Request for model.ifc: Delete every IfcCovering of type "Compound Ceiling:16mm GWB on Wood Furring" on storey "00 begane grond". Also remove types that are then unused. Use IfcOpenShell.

First a look at what the model holds.

```python
import ifcopenshell
import ifcopenshell.util.element

model = ifcopenshell.open("model.ifc")
print(model.schema)
storey = next(s for s in model.by_type("IfcBuildingStorey") if s.Name == "00 begane grond")
coverings = [e for e in ifcopenshell.util.element.get_decomposition(storey) if e.is_a("IfcCovering")]
seen = {}
for e in coverings:
    element_type = ifcopenshell.util.element.get_type(e)
    name = element_type.Name if element_type not in (None, e) else None
    seen[name] = seen.get(name, 0) + 1
for name, count in sorted(seen.items(), key=str):
    print(count, "x", name)
```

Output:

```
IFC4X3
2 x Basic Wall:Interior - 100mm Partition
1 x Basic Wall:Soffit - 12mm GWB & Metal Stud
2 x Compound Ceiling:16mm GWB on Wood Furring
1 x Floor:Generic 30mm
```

```python
import ifcopenshell
import ifcopenshell.api.root
import ifcopenshell.util.element

model = ifcopenshell.open("model.ifc")

storey = next(s for s in model.by_type("IfcBuildingStorey") if s.Name == "00 begane grond")
coverings = [e for e in ifcopenshell.util.element.get_decomposition(storey) if e.is_a("IfcCovering")]
targets = [e for e in coverings if (t := ifcopenshell.util.element.get_type(e)) not in (None, e) and t.Name == "Compound Ceiling:16mm GWB on Wood Furring"]
types = {ifcopenshell.util.element.get_type(e) for e in targets} - {None, *targets}

for e in targets:
    ifcopenshell.api.root.remove_product(model, product=e)
print(len(targets), "removed")

unused = [t for t in types if not ifcopenshell.util.element.get_types(t)]
for t in unused:
    ifcopenshell.api.root.remove_product(model, product=t)
print(len(unused), "unused types removed")

model.write("model_v2.ifc")
```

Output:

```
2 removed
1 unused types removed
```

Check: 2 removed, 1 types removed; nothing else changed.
